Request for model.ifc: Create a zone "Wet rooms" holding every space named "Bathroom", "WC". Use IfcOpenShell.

First a look at what the model holds.

```python
import ifcopenshell

model = ifcopenshell.open("model.ifc")
print(model.schema)
seen = {}
for space in model.by_type("IfcSpace"):
    seen[space.LongName] = seen.get(space.LongName, 0) + 1
for name, count in sorted(seen.items(), key=str):
    print(count, "x", name)
print("zones:", [z.Name for z in model.by_type("IfcZone")][:20])
```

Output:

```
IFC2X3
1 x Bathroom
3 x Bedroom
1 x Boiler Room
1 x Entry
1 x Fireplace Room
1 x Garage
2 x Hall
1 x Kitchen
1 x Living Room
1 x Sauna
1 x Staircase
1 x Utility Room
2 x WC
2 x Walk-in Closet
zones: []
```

```python
import ifcopenshell
import ifcopenshell.api.group
import ifcopenshell.api.root

model = ifcopenshell.open("model.ifc")

names = {"Bathroom", "WC"}
spaces = [s for s in model.by_type("IfcSpace") if s.LongName in names]

zone = ifcopenshell.api.root.create_entity(model, ifc_class="IfcZone", name="Wet rooms")
ifcopenshell.api.group.assign_group(model, products=spaces, group=zone)
print(len(spaces), "spaces in", zone.Name)

model.write("model_updated.ifc")
```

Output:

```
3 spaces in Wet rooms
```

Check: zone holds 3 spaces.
